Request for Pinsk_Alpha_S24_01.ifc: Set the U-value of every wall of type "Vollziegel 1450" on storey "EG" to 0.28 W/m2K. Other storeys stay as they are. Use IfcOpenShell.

First a look at what the model holds.

```python
import ifcopenshell
import ifcopenshell.util.element

model = ifcopenshell.open("Pinsk_Alpha_S24_01.ifc")
print(model.schema)
storey = next(s for s in model.by_type("IfcBuildingStorey") if s.Name == "EG")
walls = [e for e in ifcopenshell.util.element.get_decomposition(storey) if e.is_a("IfcWall")]
seen = {}
for e in walls:
    element_type = ifcopenshell.util.element.get_type(e)
    key = (element_type.Name if element_type != e and element_type else None, ifcopenshell.util.element.get_pset(e, "Pset_WallCommon", "ThermalTransmittance"))
    seen[key] = seen.get(key, 0) + 1
for (name, value), count in sorted(seen.items(), key=str):
    print(count, "x", name, "|", value)
```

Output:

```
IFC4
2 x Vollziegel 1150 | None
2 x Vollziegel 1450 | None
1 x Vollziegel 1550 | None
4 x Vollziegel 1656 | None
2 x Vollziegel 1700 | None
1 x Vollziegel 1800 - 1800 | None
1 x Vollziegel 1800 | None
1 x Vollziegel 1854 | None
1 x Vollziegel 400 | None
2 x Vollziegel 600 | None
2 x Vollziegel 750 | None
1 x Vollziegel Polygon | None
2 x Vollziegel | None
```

```python
import ifcopenshell
import ifcopenshell.api.pset
import ifcopenshell.util.element

model = ifcopenshell.open("Pinsk_Alpha_S24_01.ifc")

storey = next(s for s in model.by_type("IfcBuildingStorey") if s.Name == "EG")
walls = [e for e in ifcopenshell.util.element.get_decomposition(storey) if e.is_a("IfcWall")]

count = 0
for e in walls:
    element_type = ifcopenshell.util.element.get_type(e)
    if element_type in (None, e) or element_type.Name != "Vollziegel 1450":
        continue
    # add_pset returns the element's existing set when there is one.
    pset = ifcopenshell.api.pset.add_pset(model, product=e, name="Pset_WallCommon")
    ifcopenshell.api.pset.edit_pset(model, pset=pset, properties={"ThermalTransmittance": 0.28})
    count += 1

print(count, "walls updated")

model.write("Pinsk_Alpha_S24_01_updated.ifc")
```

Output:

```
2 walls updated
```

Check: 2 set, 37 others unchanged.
